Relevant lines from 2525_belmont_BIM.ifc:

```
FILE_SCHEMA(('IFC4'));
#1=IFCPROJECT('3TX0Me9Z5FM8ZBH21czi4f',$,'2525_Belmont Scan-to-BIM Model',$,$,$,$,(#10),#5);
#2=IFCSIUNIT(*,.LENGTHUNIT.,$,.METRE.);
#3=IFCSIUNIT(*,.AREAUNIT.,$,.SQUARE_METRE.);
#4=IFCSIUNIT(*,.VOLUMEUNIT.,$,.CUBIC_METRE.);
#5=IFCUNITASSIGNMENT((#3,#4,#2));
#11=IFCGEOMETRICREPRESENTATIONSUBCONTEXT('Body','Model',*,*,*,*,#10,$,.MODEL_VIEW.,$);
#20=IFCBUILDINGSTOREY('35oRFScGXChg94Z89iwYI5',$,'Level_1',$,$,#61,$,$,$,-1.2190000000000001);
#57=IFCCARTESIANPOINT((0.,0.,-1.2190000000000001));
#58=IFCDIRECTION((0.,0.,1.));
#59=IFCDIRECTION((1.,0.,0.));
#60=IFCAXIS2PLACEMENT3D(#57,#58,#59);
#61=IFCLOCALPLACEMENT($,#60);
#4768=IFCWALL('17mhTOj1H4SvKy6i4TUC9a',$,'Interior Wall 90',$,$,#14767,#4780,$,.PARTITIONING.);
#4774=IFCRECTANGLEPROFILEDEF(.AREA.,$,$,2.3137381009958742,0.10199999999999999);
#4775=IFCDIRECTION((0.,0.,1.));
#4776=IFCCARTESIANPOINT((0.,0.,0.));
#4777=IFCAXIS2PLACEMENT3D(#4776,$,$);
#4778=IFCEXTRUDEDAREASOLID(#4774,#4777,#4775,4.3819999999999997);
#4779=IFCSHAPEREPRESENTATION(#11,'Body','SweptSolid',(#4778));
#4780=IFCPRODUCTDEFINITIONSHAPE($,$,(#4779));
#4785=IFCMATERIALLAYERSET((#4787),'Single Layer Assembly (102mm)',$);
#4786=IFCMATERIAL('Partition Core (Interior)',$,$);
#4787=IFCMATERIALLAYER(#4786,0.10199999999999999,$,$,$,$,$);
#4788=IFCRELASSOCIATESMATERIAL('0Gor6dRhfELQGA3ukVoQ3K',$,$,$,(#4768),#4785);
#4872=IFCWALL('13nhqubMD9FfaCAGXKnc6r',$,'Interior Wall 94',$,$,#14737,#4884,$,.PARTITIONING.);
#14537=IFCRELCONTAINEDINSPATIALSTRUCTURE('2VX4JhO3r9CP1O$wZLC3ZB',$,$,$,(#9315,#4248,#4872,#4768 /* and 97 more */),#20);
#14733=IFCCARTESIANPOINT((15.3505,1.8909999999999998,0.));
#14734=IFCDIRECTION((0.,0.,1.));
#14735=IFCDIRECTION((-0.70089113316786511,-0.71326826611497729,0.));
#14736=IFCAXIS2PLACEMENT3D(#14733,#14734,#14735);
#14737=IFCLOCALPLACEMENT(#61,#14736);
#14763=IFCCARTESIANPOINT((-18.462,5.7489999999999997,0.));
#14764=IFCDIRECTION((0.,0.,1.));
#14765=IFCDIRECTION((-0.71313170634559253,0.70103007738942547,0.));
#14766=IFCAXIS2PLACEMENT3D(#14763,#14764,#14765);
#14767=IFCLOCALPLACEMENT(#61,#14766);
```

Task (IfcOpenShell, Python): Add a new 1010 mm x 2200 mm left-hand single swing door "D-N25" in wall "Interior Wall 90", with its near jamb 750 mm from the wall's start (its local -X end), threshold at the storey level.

```python
import numpy as np
import ifcopenshell
import ifcopenshell.api.feature
import ifcopenshell.api.geometry
import ifcopenshell.api.root
import ifcopenshell.api.spatial
import ifcopenshell.geom
import ifcopenshell.util.element
import ifcopenshell.util.placement
import ifcopenshell.util.representation
import ifcopenshell.util.shape
import ifcopenshell.util.unit

model = ifcopenshell.open("2525_belmont_BIM.ifc")
unit_scale = ifcopenshell.util.unit.calculate_unit_scale(model)
settings = ifcopenshell.geom.settings()


def volume(element):
    """Net volume in cubic metres, openings subtracted."""
    shape = ifcopenshell.geom.create_shape(settings, element)
    return ifcopenshell.util.shape.get_volume(shape.geometry)


wall = model.by_guid("17mhTOj1H4SvKy6i4TUC9a")
storey = ifcopenshell.util.element.get_container(wall, ifc_class="IfcBuildingStorey")
context = ifcopenshell.util.representation.get_context(model, "Model", "Body", "MODEL_VIEW")
before = volume(wall)

width, height, from_end, sill = 1.01, 2.2, 0.75, 0.0  # metres

# The wall runs along its own X axis, and the end named is its -X end.
wall_shape = ifcopenshell.geom.create_shape(settings, wall)
x, y, z = ifcopenshell.util.shape.get_vertices(wall_shape.geometry).T
start = x.min() + from_end
face, thickness = float(y.min()), float(y.max() - y.min())
wall_matrix = ifcopenshell.util.placement.get_local_placement(wall.ObjectPlacement)
level = ifcopenshell.util.placement.get_local_placement(storey.ObjectPlacement)[2, 3]


def in_wall(x, y):
    """Placement at x, y metres in the wall's axes, at sill height."""
    matrix = wall_matrix.copy()
    matrix[:, 3] = wall_matrix @ np.array([x / unit_scale, y / unit_scale, 0.0, 1.0])
    matrix[2, 3] = level + sill / unit_scale
    return matrix


# Opening: a box that overshoots both wall faces by 50 mm.
opening = ifcopenshell.api.root.create_entity(model, ifc_class="IfcOpeningElement", predefined_type="OPENING")
box = ifcopenshell.api.geometry.add_wall_representation(
    model, context=context, length=width, height=height, thickness=thickness + 0.1
)
ifcopenshell.api.geometry.assign_representation(model, product=opening, representation=box)
ifcopenshell.api.geometry.edit_object_placement(model, product=opening, matrix=in_wall(start, face - 0.05), is_si=False)
ifcopenshell.api.feature.add_feature(model, feature=opening, element=wall)

door = ifcopenshell.api.root.create_entity(model, ifc_class="IfcDoor", name="D-N25", predefined_type="DOOR")
door.OverallWidth, door.OverallHeight = width / unit_scale, height / unit_scale
door.OperationType = "SINGLE_SWING_LEFT"
body = ifcopenshell.api.geometry.add_door_representation(
    model,
    context=context,
    overall_width=door.OverallWidth,
    overall_height=door.OverallHeight,
    operation_type="SINGLE_SWING_LEFT",
    lining_properties={"LiningDepth": thickness / unit_scale, "ThresholdDepth": thickness / unit_scale},
)
ifcopenshell.api.geometry.assign_representation(model, product=door, representation=body)
ifcopenshell.api.spatial.assign_container(model, products=[door], relating_structure=storey)
ifcopenshell.api.feature.add_filling(model, opening=opening, element=door)

# The lining spans the wall, so the door starts at the wall face.
ifcopenshell.api.geometry.edit_object_placement(model, product=door, matrix=in_wall(start, face), is_si=False)

after = volume(wall)

print(f"wall volume {before:.3f} -> {after:.3f} m3")

model.write("2525_belmont_BIM_edited.ifc")
```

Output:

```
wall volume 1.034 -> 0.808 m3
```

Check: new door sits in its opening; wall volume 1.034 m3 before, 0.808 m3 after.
